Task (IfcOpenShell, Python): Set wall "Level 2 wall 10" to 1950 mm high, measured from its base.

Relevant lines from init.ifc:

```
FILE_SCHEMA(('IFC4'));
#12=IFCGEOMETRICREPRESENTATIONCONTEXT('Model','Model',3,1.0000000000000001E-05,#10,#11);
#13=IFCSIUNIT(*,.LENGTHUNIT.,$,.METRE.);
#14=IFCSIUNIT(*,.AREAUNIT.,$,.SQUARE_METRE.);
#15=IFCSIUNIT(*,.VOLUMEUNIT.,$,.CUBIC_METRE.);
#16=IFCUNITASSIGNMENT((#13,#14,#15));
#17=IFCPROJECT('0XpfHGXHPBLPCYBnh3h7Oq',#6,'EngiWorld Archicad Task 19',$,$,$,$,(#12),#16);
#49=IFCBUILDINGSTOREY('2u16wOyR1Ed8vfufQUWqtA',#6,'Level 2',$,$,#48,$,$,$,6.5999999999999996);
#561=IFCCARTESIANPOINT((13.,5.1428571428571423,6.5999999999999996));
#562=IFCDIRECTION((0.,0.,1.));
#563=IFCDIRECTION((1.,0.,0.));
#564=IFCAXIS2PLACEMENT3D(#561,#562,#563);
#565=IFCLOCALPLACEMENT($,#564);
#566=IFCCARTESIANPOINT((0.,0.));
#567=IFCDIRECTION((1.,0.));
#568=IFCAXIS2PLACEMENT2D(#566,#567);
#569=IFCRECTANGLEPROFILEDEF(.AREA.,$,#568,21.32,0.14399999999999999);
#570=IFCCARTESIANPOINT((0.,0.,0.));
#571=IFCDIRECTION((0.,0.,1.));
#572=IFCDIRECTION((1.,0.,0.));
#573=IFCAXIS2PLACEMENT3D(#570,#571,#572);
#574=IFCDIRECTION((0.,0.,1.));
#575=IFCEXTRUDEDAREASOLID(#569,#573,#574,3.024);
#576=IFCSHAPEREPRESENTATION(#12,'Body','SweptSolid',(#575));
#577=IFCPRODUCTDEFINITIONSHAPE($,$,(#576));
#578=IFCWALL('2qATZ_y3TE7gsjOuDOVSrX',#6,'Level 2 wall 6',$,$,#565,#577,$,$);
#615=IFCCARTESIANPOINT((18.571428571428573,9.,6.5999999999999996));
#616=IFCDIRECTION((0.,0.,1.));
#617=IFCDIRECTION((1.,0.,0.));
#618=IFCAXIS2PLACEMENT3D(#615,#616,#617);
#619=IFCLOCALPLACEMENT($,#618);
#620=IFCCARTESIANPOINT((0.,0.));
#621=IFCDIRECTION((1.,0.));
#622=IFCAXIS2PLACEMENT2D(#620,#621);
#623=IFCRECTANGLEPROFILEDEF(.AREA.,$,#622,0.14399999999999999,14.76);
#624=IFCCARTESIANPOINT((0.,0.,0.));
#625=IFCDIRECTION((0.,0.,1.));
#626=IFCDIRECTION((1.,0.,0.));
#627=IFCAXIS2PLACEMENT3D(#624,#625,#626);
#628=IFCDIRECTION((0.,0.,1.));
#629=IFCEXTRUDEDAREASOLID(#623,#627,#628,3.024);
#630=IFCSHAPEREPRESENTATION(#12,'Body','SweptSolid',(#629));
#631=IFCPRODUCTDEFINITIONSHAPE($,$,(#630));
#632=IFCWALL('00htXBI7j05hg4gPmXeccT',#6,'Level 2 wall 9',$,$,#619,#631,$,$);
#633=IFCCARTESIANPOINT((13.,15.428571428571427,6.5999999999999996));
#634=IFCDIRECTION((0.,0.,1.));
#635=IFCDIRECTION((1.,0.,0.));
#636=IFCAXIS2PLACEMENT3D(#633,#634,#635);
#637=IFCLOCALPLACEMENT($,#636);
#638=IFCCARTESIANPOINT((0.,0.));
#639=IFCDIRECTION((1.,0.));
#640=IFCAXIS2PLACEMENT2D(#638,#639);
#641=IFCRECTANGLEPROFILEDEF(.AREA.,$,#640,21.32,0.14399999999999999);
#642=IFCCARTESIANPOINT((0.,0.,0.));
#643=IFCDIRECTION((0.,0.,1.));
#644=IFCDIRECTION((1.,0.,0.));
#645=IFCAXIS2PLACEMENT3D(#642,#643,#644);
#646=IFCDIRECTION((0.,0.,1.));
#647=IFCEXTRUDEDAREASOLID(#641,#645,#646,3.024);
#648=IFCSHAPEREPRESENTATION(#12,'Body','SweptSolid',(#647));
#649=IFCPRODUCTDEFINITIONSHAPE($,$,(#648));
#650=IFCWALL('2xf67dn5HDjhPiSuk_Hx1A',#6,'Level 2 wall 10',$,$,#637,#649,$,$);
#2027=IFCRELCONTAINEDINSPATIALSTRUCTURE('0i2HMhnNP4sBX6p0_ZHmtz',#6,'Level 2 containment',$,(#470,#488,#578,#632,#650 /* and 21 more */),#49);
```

```python
import ifcopenshell
import ifcopenshell.geom
import ifcopenshell.util.shape
import ifcopenshell.util.unit

model = ifcopenshell.open("init.ifc")
unit_scale = ifcopenshell.util.unit.calculate_unit_scale(model)
settings = ifcopenshell.geom.settings()


def volume(element):
    """Net volume in cubic metres, openings subtracted."""
    shape = ifcopenshell.geom.create_shape(settings, element)
    return ifcopenshell.util.shape.get_volume(shape.geometry)


wall = model.by_guid("2xf67dn5HDjhPiSuk_Hx1A")
before = volume(wall)

body = next(r for r in wall.Representation.Representations if r.RepresentationIdentifier == "Body")
solid = body.Items[0]
old_height = solid.Depth
solid.Depth = 1.95 / unit_scale
after = volume(wall)

print(f"height {old_height:g} -> {solid.Depth:g}, volume {before:.3f} -> {after:.3f} m3")

model.write("init_rev.ifc")
```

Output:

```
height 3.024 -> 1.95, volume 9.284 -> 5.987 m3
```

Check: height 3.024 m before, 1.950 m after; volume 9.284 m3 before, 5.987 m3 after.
